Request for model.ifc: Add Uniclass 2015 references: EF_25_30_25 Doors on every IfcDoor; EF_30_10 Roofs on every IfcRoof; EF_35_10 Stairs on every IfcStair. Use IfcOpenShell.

First a look at what the model holds.

```python
import ifcopenshell

model = ifcopenshell.open("model.ifc")
print(model.schema)
print("classifications:", [c.Name for c in model.by_type("IfcClassification")])
for ifc_class in ("IfcDoor", "IfcRoof", "IfcStair", "IfcWall", "IfcWindow"):
    print(ifc_class, len(model.by_type(ifc_class)))
```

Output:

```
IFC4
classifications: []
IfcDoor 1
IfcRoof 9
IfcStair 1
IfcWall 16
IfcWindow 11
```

```python
import ifcopenshell
import ifcopenshell.api.classification

model = ifcopenshell.open("model.ifc")

system = ifcopenshell.api.classification.add_classification(model, classification="Uniclass 2015")

codes = {
    "IfcDoor": ("EF_25_30_25", "Doors"),
    "IfcRoof": ("EF_30_10", "Roofs"),
    "IfcStair": ("EF_35_10", "Stairs"),
}
for ifc_class, (code, name) in codes.items():
    products = model.by_type(ifc_class)
    ifcopenshell.api.classification.add_reference(
        model, products=products, classification=system, identification=code, name=name
    )
    print(code, len(products))

model.write("model-out.ifc")
```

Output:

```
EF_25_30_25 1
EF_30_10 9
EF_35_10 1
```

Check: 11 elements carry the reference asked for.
